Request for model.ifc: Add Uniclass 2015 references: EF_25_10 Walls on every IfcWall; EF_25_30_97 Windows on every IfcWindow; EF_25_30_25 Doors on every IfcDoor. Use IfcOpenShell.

First a look at what the model holds.

```python
import ifcopenshell

model = ifcopenshell.open("model.ifc")
print(model.schema)
print("classifications:", [c.Name for c in model.by_type("IfcClassification")])
for ifc_class in ("IfcDoor", "IfcRoof", "IfcStair", "IfcWall", "IfcWindow"):
    print(ifc_class, len(model.by_type(ifc_class)))
```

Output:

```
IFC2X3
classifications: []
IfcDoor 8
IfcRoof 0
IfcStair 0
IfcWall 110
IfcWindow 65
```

```python
import ifcopenshell
import ifcopenshell.api.classification

model = ifcopenshell.open("model.ifc")

# IFC2X3 requires Source and Edition and has no link from the project to the system.
system = model.create_entity("IfcClassification", Source="NBS", Edition="2015", Name="Uniclass 2015")

codes = {
    "IfcWall": ("EF_25_10", "Walls"),
    "IfcWindow": ("EF_25_30_97", "Windows"),
    "IfcDoor": ("EF_25_30_25", "Doors"),
}
for ifc_class, (code, name) in codes.items():
    products = model.by_type(ifc_class)
    ifcopenshell.api.classification.add_reference(
        model, products=products, classification=system, identification=code, name=name
    )
    print(code, len(products))

model.write("model_v2.ifc")
```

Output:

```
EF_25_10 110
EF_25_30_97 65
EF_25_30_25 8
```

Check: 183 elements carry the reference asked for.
